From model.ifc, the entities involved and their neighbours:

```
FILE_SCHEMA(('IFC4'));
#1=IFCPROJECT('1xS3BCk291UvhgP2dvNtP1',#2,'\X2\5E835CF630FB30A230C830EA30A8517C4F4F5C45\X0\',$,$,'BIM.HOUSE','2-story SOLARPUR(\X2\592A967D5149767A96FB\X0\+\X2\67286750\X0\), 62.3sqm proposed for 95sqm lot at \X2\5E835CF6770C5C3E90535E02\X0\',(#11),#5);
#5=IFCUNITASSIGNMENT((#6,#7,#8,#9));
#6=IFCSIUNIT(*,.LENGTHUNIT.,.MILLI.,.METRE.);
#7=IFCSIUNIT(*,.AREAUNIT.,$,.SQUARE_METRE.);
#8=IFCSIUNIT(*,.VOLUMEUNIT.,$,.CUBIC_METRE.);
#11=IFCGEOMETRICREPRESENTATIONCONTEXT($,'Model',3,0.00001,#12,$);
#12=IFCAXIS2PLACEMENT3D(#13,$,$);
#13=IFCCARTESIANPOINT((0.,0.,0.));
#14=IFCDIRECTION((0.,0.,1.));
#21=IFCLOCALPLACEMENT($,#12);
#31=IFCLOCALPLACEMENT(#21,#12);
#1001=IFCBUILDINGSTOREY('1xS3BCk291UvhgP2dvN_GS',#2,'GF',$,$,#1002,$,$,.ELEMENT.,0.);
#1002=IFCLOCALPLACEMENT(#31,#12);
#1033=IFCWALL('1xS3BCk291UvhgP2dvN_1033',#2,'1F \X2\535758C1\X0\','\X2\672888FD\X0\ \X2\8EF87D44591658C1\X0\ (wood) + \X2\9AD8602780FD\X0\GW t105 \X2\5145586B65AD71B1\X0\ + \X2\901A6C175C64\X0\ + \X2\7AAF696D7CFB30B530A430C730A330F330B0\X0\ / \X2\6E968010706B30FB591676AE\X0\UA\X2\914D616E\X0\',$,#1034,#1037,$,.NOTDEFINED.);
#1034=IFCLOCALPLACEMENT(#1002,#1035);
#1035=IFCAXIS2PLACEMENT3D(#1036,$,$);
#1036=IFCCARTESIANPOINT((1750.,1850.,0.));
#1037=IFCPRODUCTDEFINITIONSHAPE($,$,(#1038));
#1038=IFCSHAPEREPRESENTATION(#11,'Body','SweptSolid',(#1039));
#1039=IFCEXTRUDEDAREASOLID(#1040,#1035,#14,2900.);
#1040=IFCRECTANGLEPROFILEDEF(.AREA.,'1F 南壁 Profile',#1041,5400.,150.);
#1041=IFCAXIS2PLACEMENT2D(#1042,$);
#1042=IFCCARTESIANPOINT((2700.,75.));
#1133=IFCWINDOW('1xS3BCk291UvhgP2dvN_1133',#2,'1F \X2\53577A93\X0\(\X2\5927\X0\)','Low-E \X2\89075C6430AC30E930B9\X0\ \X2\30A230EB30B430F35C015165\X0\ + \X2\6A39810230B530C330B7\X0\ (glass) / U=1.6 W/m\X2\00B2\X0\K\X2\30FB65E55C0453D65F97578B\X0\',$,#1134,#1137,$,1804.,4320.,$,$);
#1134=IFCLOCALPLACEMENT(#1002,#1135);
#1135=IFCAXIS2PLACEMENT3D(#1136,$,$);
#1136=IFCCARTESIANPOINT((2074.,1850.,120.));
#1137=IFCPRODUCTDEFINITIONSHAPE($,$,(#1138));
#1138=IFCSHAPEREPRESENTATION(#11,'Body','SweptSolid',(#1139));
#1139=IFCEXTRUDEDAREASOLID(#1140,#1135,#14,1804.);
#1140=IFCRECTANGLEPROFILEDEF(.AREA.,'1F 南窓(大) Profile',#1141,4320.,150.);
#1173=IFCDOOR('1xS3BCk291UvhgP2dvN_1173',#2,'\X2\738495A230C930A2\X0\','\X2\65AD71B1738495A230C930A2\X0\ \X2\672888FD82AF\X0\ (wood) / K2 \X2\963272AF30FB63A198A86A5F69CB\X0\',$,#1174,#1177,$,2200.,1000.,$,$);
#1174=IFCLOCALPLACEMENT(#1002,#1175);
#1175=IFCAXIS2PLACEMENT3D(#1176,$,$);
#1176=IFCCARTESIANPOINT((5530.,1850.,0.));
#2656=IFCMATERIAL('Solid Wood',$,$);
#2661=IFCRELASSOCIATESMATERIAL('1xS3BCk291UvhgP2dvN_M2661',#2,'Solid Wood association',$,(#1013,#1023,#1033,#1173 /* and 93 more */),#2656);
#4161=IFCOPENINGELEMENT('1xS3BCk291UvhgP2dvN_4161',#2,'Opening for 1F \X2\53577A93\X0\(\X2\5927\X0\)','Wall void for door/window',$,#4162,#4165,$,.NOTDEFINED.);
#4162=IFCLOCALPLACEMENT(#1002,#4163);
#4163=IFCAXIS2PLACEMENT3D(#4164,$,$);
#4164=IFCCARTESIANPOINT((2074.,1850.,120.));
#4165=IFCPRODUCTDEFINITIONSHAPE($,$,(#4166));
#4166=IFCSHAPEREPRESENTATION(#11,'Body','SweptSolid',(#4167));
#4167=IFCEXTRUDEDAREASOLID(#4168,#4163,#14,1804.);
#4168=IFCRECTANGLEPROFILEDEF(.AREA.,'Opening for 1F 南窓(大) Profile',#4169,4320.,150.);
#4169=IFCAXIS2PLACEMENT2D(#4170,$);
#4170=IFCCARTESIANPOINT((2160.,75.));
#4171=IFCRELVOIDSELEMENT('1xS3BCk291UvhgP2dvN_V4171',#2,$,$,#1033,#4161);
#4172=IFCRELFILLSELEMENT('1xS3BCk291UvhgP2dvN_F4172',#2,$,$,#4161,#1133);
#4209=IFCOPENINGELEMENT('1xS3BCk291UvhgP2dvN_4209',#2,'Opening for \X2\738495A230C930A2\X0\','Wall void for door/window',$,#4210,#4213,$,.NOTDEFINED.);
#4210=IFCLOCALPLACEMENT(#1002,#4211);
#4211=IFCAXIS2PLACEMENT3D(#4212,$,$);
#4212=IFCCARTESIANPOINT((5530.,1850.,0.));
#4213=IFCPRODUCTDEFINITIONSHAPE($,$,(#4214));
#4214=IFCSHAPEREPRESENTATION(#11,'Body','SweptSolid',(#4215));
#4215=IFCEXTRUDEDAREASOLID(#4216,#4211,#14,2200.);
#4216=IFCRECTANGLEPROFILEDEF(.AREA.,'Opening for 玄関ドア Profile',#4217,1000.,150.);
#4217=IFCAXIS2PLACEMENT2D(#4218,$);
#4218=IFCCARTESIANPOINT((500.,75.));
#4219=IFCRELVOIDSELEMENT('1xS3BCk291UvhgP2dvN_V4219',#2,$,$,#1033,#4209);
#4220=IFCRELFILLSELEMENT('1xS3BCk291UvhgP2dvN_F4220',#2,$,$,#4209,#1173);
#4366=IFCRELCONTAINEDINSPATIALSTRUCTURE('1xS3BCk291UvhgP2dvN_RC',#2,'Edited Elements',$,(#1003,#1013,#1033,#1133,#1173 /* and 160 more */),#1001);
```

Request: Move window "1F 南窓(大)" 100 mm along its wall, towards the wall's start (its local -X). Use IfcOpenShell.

```python
import ifcopenshell
import ifcopenshell.api.geometry
import ifcopenshell.util.placement
import ifcopenshell.util.unit

model = ifcopenshell.open("model.ifc")
unit_scale = ifcopenshell.util.unit.calculate_unit_scale(model)

window = model.by_guid("1xS3BCk291UvhgP2dvN_1133")
opening = window.FillsVoids[0].RelatingOpeningElement
wall = opening.VoidsElements[0].RelatingBuildingElement

wall_matrix = ifcopenshell.util.placement.get_local_placement(wall.ObjectPlacement)
shift = wall_matrix[:3, 0] * -0.1 / unit_scale
before = ifcopenshell.util.placement.get_local_placement(window.ObjectPlacement)[:3, 3].copy()

# The window is not placed relative to its opening, so move both.
for product in (opening, window):
    matrix = ifcopenshell.util.placement.get_local_placement(product.ObjectPlacement)
    matrix[:3, 3] += shift
    ifcopenshell.api.geometry.edit_object_placement(model, product=product, matrix=matrix, is_si=False)

after = ifcopenshell.util.placement.get_local_placement(window.ObjectPlacement)[:3, 3]
print("window moved by", (after - before).round(3) + 0.0)

model.write("model_edited.ifc")
```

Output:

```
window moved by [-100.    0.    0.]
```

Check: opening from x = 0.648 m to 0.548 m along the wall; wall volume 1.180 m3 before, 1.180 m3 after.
